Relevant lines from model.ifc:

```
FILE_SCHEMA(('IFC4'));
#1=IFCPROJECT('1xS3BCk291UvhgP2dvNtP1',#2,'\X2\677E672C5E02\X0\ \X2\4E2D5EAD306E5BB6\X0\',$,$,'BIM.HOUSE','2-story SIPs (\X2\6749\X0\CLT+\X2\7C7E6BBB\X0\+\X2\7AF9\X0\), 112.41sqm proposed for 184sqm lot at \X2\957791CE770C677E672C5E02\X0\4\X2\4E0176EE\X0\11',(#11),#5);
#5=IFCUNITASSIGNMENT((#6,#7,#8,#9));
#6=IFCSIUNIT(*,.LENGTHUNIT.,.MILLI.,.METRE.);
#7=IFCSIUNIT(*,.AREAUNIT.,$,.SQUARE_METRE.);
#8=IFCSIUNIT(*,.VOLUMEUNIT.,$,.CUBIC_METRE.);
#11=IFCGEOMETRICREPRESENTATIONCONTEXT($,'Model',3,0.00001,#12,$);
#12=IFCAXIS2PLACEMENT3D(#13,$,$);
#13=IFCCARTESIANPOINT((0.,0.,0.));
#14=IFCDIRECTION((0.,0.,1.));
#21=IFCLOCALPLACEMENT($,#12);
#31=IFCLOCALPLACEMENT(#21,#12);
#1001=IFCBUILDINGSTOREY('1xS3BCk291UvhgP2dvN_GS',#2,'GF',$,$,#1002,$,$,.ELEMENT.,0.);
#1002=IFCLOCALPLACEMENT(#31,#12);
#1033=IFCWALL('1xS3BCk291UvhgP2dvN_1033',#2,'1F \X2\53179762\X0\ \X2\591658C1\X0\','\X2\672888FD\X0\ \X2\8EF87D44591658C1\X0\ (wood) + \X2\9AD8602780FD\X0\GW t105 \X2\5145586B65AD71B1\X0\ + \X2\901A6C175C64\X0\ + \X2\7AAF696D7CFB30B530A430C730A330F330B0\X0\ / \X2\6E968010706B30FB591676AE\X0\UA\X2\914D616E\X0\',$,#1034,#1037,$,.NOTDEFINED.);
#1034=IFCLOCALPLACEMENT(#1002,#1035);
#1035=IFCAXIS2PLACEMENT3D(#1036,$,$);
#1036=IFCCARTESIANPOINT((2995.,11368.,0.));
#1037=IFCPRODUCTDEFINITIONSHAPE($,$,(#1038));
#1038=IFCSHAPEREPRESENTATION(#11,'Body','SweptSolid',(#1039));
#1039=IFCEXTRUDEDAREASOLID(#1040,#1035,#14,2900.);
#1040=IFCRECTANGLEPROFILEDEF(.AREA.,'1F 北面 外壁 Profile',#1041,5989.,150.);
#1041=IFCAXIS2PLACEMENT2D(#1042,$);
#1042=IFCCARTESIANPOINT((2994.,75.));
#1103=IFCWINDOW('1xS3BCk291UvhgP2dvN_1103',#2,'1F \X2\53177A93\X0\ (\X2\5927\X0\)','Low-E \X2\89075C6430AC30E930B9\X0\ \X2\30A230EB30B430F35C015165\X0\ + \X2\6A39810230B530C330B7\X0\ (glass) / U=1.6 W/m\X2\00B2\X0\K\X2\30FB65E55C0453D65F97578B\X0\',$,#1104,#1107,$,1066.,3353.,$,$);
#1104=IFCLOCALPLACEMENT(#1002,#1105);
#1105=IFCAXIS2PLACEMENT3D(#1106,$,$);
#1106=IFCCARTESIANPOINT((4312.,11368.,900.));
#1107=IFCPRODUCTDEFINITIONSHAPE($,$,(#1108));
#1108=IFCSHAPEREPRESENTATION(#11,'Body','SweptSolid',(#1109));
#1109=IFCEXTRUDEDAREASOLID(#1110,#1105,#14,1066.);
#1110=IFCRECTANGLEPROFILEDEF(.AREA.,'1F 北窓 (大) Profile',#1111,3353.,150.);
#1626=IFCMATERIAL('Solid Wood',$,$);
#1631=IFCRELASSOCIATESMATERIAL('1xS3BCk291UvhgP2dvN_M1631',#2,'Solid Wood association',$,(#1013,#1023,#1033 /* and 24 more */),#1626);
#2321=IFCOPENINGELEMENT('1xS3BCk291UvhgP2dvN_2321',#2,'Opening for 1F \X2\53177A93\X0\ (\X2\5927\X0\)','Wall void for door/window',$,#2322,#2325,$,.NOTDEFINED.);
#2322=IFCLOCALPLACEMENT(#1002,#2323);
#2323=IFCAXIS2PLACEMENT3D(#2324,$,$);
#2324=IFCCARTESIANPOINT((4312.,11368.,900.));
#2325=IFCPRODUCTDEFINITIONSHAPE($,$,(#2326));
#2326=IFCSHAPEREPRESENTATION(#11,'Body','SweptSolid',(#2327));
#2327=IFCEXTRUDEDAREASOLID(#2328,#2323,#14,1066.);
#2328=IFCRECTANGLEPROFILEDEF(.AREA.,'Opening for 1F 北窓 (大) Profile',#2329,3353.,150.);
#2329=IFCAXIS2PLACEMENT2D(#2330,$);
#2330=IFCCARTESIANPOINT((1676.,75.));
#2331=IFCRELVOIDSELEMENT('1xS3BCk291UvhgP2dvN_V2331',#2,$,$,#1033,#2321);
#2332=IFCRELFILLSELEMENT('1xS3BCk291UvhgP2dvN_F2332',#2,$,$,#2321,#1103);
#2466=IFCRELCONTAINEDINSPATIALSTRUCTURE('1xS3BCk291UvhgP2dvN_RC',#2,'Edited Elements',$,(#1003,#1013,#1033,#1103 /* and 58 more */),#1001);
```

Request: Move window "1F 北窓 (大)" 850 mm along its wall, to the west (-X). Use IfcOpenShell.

```python
import ifcopenshell
import ifcopenshell.api.geometry
import ifcopenshell.util.placement
import ifcopenshell.util.unit

model = ifcopenshell.open("model.ifc")
unit_scale = ifcopenshell.util.unit.calculate_unit_scale(model)

window = model.by_guid("1xS3BCk291UvhgP2dvN_1103")
opening = window.FillsVoids[0].RelatingOpeningElement
wall = opening.VoidsElements[0].RelatingBuildingElement

wall_matrix = ifcopenshell.util.placement.get_local_placement(wall.ObjectPlacement)
shift = wall_matrix[:3, 0] * -0.85 / unit_scale
before = ifcopenshell.util.placement.get_local_placement(window.ObjectPlacement)[:3, 3].copy()

# The window is not placed relative to its opening, so move both.
for product in (opening, window):
    matrix = ifcopenshell.util.placement.get_local_placement(product.ObjectPlacement)
    matrix[:3, 3] += shift
    ifcopenshell.api.geometry.edit_object_placement(model, product=product, matrix=matrix, is_si=False)

after = ifcopenshell.util.placement.get_local_placement(window.ObjectPlacement)[:3, 3]
print("window moved by", (after - before).round(3) + 0.0)

model.write("model-out.ifc")
```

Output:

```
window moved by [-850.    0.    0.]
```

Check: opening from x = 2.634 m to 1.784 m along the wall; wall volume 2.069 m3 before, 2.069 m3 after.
